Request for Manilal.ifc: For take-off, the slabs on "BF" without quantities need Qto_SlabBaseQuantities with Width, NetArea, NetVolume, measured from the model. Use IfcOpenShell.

First a look at what the model holds.

```python
import ifcopenshell
import ifcopenshell.util.element
import ifcopenshell.util.unit

model = ifcopenshell.open("Manilal.ifc")
print(model.schema)
for unit_type in ("LENGTHUNIT", "AREAUNIT", "VOLUMEUNIT"):
    print(unit_type, ifcopenshell.util.unit.calculate_unit_scale(model, unit_type))
storey = next(s for s in model.by_type("IfcBuildingStorey") if s.Name == "BF")
slabs = [e for e in ifcopenshell.util.element.get_decomposition(storey) if e.is_a("IfcSlab")]
for e in sorted(slabs, key=lambda e: e.id()):
    print(e.id(), e.is_a(), e.Name, list(ifcopenshell.util.element.get_psets(e, qtos_only=True)), sep=" | ")
```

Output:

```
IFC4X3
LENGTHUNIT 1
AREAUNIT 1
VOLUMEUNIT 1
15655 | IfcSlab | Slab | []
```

```python
import ifcopenshell
import ifcopenshell.api.pset
import ifcopenshell.geom
import ifcopenshell.util.element
import ifcopenshell.util.shape
import ifcopenshell.util.unit

model = ifcopenshell.open("Manilal.ifc")
unit_scale = ifcopenshell.util.unit.calculate_unit_scale(model)
area_scale = ifcopenshell.util.unit.calculate_unit_scale(model, "AREAUNIT")
volume_scale = ifcopenshell.util.unit.calculate_unit_scale(model, "VOLUMEUNIT")
settings = ifcopenshell.geom.settings()

storey = next(s for s in model.by_type("IfcBuildingStorey") if s.Name == "BF")
slabs = [e for e in ifcopenshell.util.element.get_decomposition(storey) if e.is_a("IfcSlab")]

for e in sorted(slabs, key=lambda e: e.id()):
    if ifcopenshell.util.element.get_psets(e, qtos_only=True, should_inherit=False):
        continue
    # Geometry comes back in metres, in the element's own axes.
    shape = ifcopenshell.geom.create_shape(settings, e)
    values = {
        "Width": ifcopenshell.util.shape.get_z(shape.geometry) / unit_scale,
        "NetArea": ifcopenshell.util.shape.get_footprint_area(shape.geometry) / area_scale,
        "NetVolume": ifcopenshell.util.shape.get_volume(shape.geometry) / volume_scale,
    }
    qto = ifcopenshell.api.pset.add_qto(model, product=e, name="Qto_SlabBaseQuantities")
    ifcopenshell.api.pset.edit_qto(model, qto=qto, properties=values)
    print(e.id(), {k: round(v, 3) for k, v in values.items()})

model.write("Manilal_v2.ifc")
```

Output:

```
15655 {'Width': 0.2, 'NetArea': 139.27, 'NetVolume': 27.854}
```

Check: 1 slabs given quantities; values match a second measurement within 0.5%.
